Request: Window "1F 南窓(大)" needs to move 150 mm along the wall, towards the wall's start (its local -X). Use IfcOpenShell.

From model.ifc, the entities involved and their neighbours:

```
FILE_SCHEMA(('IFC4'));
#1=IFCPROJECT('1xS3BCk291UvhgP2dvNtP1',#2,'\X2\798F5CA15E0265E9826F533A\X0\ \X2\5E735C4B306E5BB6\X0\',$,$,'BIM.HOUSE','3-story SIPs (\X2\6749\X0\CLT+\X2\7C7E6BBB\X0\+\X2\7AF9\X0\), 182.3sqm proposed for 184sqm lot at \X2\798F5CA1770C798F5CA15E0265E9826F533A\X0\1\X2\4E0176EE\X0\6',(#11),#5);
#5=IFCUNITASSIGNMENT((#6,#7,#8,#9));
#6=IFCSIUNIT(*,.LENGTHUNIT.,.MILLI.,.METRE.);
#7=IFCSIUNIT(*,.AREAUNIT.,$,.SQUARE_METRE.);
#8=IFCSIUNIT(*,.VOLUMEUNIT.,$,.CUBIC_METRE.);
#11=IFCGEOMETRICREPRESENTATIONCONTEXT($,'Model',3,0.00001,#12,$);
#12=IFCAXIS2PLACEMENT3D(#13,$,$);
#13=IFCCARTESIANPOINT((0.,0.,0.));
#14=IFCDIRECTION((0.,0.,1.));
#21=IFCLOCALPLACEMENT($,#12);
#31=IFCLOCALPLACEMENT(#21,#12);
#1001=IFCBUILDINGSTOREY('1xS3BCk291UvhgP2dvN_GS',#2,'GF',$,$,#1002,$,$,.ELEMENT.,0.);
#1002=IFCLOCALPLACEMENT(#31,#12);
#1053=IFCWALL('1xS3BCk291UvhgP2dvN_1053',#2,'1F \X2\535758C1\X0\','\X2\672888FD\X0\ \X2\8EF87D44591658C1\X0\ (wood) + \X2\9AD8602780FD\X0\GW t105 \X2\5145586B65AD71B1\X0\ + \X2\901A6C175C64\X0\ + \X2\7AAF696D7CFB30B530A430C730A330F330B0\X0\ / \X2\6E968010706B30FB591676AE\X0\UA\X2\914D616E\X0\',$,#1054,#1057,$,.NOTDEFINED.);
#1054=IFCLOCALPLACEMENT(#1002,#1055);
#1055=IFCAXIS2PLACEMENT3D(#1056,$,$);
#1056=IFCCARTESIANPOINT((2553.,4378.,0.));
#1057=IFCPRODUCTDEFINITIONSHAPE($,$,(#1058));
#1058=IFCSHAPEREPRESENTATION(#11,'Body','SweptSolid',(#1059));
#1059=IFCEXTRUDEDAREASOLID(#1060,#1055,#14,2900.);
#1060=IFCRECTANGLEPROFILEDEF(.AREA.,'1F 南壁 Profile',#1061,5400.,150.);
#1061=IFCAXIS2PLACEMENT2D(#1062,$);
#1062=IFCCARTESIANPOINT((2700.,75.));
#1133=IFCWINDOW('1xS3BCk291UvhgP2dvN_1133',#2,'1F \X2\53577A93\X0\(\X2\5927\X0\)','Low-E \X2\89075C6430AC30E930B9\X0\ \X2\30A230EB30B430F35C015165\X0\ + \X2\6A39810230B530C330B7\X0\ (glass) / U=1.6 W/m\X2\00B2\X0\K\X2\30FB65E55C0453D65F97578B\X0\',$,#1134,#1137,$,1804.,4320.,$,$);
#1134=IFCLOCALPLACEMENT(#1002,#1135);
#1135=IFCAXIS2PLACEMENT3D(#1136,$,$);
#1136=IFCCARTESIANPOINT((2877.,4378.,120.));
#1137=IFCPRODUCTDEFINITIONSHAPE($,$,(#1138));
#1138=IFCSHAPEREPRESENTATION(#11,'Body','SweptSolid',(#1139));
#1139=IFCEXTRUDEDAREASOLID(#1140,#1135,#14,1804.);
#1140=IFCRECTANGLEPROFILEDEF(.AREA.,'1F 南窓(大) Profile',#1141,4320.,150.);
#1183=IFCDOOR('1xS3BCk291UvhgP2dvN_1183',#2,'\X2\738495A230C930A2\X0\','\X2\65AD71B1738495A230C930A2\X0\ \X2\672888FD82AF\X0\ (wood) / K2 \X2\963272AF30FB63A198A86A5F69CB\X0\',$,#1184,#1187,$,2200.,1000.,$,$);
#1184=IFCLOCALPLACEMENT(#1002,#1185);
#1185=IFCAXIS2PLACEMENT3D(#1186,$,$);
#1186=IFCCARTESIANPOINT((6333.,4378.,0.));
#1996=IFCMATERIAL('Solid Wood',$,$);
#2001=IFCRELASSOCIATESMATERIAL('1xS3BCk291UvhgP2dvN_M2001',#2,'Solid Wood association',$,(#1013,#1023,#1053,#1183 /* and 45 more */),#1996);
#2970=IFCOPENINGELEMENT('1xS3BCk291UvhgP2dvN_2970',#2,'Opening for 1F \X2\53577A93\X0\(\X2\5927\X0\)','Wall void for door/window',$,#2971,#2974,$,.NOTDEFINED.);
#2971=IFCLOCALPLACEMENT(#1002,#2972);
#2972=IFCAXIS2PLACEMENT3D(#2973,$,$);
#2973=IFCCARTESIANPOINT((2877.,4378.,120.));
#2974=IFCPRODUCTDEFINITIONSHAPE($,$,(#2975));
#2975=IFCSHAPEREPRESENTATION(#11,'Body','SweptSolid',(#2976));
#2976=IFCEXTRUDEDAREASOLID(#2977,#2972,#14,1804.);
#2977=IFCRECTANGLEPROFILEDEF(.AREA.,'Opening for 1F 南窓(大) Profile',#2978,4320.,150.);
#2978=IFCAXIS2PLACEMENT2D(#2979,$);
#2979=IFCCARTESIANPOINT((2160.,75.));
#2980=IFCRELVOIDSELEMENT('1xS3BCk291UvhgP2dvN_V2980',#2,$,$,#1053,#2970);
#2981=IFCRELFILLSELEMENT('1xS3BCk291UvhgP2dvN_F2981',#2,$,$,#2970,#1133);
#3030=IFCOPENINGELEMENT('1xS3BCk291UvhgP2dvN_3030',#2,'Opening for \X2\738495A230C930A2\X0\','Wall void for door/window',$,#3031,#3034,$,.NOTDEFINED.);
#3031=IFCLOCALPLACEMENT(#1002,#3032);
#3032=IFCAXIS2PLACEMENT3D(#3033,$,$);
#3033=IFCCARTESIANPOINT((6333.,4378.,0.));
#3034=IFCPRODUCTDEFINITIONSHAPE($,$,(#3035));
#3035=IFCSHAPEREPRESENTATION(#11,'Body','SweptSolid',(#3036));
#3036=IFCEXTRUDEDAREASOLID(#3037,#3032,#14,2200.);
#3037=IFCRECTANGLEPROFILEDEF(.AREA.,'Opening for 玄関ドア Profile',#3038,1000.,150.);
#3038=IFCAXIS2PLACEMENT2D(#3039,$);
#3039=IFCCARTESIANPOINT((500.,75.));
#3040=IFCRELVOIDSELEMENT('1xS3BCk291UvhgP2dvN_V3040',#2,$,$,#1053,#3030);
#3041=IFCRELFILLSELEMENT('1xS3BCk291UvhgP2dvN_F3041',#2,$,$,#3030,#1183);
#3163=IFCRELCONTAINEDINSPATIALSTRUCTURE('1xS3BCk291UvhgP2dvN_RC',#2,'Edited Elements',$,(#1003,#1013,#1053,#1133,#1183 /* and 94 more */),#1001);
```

```python
import ifcopenshell
import ifcopenshell.api.geometry
import ifcopenshell.util.placement

model = ifcopenshell.open("model.ifc")

window = model.by_id(1133)
opening = window.FillsVoids[0].RelatingOpeningElement
wall = opening.VoidsElements[0].RelatingBuildingElement

wall_matrix = ifcopenshell.util.placement.get_local_placement(wall.ObjectPlacement)
shift = wall_matrix[:3, 0] * -150.0
before = ifcopenshell.util.placement.get_local_placement(window.ObjectPlacement)[:3, 3].copy()

# The window is not placed relative to its opening, so move both.
for product in (opening, window):
    matrix = ifcopenshell.util.placement.get_local_placement(product.ObjectPlacement)
    matrix[:3, 3] += shift
    ifcopenshell.api.geometry.edit_object_placement(model, product=product, matrix=matrix, is_si=False)

after = ifcopenshell.util.placement.get_local_placement(window.ObjectPlacement)[:3, 3]
print("window moved by", (after - before).round(3) + 0.0)

model.write("model_v2.ifc")
```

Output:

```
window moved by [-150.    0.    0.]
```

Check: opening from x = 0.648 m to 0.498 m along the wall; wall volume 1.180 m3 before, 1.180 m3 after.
